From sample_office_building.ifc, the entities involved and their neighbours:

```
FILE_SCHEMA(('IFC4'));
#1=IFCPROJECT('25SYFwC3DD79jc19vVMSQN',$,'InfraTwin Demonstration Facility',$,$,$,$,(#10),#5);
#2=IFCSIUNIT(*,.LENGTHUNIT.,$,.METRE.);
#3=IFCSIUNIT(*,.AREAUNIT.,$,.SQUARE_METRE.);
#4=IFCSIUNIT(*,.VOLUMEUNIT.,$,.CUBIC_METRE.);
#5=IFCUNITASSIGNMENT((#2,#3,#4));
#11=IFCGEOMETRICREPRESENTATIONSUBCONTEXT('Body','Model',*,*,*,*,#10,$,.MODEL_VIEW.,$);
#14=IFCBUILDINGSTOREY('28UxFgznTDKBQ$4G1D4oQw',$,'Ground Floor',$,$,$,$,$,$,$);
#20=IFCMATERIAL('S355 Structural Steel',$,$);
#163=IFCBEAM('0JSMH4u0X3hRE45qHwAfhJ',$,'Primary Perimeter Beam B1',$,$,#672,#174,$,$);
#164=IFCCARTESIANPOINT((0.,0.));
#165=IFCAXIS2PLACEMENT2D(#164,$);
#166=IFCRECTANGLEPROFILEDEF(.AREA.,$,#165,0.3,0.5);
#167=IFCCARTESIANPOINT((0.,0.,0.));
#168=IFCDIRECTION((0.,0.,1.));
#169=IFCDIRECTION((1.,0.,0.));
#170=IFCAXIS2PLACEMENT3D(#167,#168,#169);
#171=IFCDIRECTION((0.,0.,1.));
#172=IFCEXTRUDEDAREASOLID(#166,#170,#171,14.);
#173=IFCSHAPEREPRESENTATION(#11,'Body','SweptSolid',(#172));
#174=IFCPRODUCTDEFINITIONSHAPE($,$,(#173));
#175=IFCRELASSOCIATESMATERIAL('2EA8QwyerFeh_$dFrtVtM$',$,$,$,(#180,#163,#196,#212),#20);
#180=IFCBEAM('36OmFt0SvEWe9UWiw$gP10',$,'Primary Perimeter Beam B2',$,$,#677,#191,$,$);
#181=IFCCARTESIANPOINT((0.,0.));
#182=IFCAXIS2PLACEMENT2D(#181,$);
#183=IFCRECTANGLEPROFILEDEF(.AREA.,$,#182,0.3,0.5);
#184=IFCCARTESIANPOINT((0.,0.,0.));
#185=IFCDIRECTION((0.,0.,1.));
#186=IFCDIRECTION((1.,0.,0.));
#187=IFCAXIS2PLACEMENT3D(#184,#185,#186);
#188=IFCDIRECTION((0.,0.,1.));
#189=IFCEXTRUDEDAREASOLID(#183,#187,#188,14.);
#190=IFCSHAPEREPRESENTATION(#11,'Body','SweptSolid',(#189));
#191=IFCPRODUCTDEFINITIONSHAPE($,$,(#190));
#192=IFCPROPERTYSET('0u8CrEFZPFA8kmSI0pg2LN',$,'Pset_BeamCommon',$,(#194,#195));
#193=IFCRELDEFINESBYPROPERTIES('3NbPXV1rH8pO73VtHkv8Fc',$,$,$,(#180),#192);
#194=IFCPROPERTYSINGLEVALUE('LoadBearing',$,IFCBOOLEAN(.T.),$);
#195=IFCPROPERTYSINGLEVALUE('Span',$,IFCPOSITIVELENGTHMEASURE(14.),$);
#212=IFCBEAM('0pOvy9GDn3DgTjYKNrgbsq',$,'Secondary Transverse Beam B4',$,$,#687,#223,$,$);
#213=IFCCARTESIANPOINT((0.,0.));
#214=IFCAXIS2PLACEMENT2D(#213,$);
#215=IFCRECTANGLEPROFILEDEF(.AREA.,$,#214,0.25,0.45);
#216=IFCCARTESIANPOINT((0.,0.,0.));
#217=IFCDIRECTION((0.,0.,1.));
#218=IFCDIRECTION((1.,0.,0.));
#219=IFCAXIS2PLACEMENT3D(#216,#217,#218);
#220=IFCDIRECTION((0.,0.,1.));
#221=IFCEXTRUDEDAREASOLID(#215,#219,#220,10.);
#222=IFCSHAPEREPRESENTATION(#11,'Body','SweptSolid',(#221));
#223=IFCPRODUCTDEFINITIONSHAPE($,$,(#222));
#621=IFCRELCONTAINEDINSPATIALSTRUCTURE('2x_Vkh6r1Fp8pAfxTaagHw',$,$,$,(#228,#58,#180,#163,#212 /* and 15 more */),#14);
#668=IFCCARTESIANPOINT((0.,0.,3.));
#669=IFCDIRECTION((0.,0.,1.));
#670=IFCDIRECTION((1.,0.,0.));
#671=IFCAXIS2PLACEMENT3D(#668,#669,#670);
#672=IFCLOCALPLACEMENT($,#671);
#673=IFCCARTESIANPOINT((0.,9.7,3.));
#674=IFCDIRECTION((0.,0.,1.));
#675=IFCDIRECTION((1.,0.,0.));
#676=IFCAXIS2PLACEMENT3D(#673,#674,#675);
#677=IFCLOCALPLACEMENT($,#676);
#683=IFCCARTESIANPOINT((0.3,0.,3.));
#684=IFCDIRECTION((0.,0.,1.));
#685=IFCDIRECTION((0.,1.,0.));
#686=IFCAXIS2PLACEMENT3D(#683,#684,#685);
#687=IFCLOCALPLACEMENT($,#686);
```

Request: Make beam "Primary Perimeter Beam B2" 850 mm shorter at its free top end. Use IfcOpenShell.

```python
import ifcopenshell
import ifcopenshell.api.pset
import ifcopenshell.util.element
import ifcopenshell.util.representation
import ifcopenshell.util.unit

model = ifcopenshell.open("sample_office_building.ifc")
unit_scale = ifcopenshell.util.unit.calculate_unit_scale(model)

member = model.by_guid("36OmFt0SvEWe9UWiw$gP10")
change = -0.85 / unit_scale

# The extrusion runs towards the end named, so only its depth changes.
body = ifcopenshell.util.representation.get_representation(member, "Model", "Body")
solid = body.Items[0]
old_length = solid.Depth
solid.Depth += change

# Update the stored length and volume.
pset = model.by_id(ifcopenshell.util.element.get_pset(member, "Pset_BeamCommon", should_inherit=False)["id"])
ifcopenshell.api.pset.edit_pset(model, pset=pset, properties={
    "Span": model.create_entity("IfcPositiveLengthMeasure", solid.Depth),
})

print(f"length {old_length:g} -> {solid.Depth:g}")

model.write("sample_office_building_rev.ifc")
```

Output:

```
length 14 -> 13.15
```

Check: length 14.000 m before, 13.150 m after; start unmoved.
